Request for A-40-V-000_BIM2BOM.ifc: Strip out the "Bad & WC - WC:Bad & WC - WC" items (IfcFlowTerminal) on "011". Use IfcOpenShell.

First a look at what the model holds.

```python
import ifcopenshell
import ifcopenshell.util.element

model = ifcopenshell.open("A-40-V-000_BIM2BOM.ifc")
print(model.schema)
storey = next(s for s in model.by_type("IfcBuildingStorey") if s.Name == "011")
terminals = [e for e in ifcopenshell.util.element.get_decomposition(storey) if e.is_a("IfcFlowTerminal")]
seen = {}
for e in terminals:
    element_type = ifcopenshell.util.element.get_type(e)
    name = element_type.Name if element_type not in (None, e) else None
    seen[name] = seen.get(name, 0) + 1
for name, count in sorted(seen.items(), key=str):
    print(count, "x", name)
```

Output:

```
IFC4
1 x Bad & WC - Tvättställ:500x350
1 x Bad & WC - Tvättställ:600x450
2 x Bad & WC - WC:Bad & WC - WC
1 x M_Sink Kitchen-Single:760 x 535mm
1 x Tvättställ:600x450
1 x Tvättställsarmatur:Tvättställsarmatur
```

```python
import ifcopenshell
import ifcopenshell.api.root
import ifcopenshell.util.element

model = ifcopenshell.open("A-40-V-000_BIM2BOM.ifc")

storey = next(s for s in model.by_type("IfcBuildingStorey") if s.Name == "011")
terminals = [e for e in ifcopenshell.util.element.get_decomposition(storey) if e.is_a("IfcFlowTerminal")]
targets = [e for e in terminals if (t := ifcopenshell.util.element.get_type(e)) not in (None, e) and t.Name == "Bad & WC - WC:Bad & WC - WC"]

for e in targets:
    ifcopenshell.api.root.remove_product(model, product=e)
print(len(targets), "removed")

model.write("A-40-V-000_BIM2BOM_v2.ifc")
```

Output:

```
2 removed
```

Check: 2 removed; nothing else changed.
